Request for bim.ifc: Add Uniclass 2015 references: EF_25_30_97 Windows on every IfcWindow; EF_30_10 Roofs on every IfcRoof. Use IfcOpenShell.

First a look at what the model holds.

```python
import ifcopenshell

model = ifcopenshell.open("bim.ifc")
print(model.schema)
print("classifications:", [c.Name for c in model.by_type("IfcClassification")])
for ifc_class in ("IfcDoor", "IfcRoof", "IfcStair", "IfcWall", "IfcWindow"):
    print(ifc_class, len(model.by_type(ifc_class)))
```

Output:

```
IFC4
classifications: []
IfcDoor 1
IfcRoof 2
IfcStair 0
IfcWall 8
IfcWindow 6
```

```python
import ifcopenshell
import ifcopenshell.api.classification

model = ifcopenshell.open("bim.ifc")

system = ifcopenshell.api.classification.add_classification(model, classification="Uniclass 2015")

codes = {
    "IfcWindow": ("EF_25_30_97", "Windows"),
    "IfcRoof": ("EF_30_10", "Roofs"),
}
for ifc_class, (code, name) in codes.items():
    products = model.by_type(ifc_class)
    ifcopenshell.api.classification.add_reference(
        model, products=products, classification=system, identification=code, name=name
    )
    print(code, len(products))

model.write("bim_edited.ifc")
```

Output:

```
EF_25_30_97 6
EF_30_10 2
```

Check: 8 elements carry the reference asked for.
